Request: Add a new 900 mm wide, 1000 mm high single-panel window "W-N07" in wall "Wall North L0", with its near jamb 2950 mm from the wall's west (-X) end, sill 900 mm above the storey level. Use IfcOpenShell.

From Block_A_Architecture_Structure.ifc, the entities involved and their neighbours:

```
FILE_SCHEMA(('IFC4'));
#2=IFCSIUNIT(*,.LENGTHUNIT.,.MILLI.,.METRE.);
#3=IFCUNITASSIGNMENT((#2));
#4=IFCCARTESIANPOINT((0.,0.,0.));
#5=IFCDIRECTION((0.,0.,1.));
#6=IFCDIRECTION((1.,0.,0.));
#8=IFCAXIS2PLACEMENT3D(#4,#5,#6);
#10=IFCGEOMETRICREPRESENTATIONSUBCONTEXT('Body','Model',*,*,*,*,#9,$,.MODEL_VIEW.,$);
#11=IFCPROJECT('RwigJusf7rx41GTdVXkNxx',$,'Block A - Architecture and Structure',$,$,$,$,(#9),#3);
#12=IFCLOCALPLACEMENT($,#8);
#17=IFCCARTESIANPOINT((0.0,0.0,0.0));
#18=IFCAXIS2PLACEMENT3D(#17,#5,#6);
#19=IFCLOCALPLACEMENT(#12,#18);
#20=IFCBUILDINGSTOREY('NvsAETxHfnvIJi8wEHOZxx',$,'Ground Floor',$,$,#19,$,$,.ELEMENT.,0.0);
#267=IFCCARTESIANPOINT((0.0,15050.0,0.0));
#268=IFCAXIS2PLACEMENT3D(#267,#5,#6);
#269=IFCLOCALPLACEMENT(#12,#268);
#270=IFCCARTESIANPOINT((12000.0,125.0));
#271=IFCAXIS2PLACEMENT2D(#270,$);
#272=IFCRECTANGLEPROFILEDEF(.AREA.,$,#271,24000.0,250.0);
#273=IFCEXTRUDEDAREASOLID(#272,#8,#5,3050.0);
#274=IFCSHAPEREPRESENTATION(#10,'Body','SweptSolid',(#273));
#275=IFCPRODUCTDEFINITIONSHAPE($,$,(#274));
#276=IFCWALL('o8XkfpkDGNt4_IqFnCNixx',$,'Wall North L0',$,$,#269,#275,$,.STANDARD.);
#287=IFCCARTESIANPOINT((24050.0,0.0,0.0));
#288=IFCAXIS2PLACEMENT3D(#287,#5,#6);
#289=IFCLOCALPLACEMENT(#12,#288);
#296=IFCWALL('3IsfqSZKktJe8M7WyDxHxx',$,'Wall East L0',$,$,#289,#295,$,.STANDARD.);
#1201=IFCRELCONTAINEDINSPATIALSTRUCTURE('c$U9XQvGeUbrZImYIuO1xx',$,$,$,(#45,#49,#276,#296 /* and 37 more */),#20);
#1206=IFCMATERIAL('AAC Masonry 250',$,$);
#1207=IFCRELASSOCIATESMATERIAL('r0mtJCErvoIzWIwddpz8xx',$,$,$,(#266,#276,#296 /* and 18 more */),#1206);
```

```python
import numpy as np
import ifcopenshell
import ifcopenshell.api.feature
import ifcopenshell.api.geometry
import ifcopenshell.api.root
import ifcopenshell.api.spatial
import ifcopenshell.geom
import ifcopenshell.util.element
import ifcopenshell.util.placement
import ifcopenshell.util.representation
import ifcopenshell.util.shape
import ifcopenshell.util.unit

model = ifcopenshell.open("Block_A_Architecture_Structure.ifc")
unit_scale = ifcopenshell.util.unit.calculate_unit_scale(model)
settings = ifcopenshell.geom.settings()


def volume(element):
    """Net volume in cubic metres, openings subtracted."""
    shape = ifcopenshell.geom.create_shape(settings, element)
    return ifcopenshell.util.shape.get_volume(shape.geometry)


wall = model.by_guid("o8XkfpkDGNt4_IqFnCNixx")
storey = ifcopenshell.util.element.get_container(wall, ifc_class="IfcBuildingStorey")
context = ifcopenshell.util.representation.get_context(model, "Model", "Body", "MODEL_VIEW")
before = volume(wall)

width, height, from_end, sill = 0.9, 1, 2.95, 0.9  # metres

# The wall runs along its own X axis, and the end named is its -X end.
wall_shape = ifcopenshell.geom.create_shape(settings, wall)
x, y, z = ifcopenshell.util.shape.get_vertices(wall_shape.geometry).T
start = x.min() + from_end
face, thickness = float(y.min()), float(y.max() - y.min())
wall_matrix = ifcopenshell.util.placement.get_local_placement(wall.ObjectPlacement)
level = ifcopenshell.util.placement.get_local_placement(storey.ObjectPlacement)[2, 3]


def in_wall(x, y):
    """Placement at x, y metres in the wall's axes, at sill height."""
    matrix = wall_matrix.copy()
    matrix[:, 3] = wall_matrix @ np.array([x / unit_scale, y / unit_scale, 0.0, 1.0])
    matrix[2, 3] = level + sill / unit_scale
    return matrix


# Opening: a box that overshoots both wall faces by 50 mm.
opening = ifcopenshell.api.root.create_entity(model, ifc_class="IfcOpeningElement", predefined_type="OPENING")
box = ifcopenshell.api.geometry.add_wall_representation(
    model, context=context, length=width, height=height, thickness=thickness + 0.1
)
ifcopenshell.api.geometry.assign_representation(model, product=opening, representation=box)
ifcopenshell.api.geometry.edit_object_placement(model, product=opening, matrix=in_wall(start, face - 0.05), is_si=False)
ifcopenshell.api.feature.add_feature(model, feature=opening, element=wall)

window = ifcopenshell.api.root.create_entity(model, ifc_class="IfcWindow", name="W-N07", predefined_type="WINDOW")
window.OverallWidth, window.OverallHeight = width / unit_scale, height / unit_scale
window.PartitioningType = "SINGLE_PANEL"
body = ifcopenshell.api.geometry.add_window_representation(
    model,
    context=context,
    overall_width=window.OverallWidth,
    overall_height=window.OverallHeight,
    partition_type="SINGLE_PANEL",
)
ifcopenshell.api.geometry.assign_representation(model, product=window, representation=body)
ifcopenshell.api.spatial.assign_container(model, products=[window], relating_structure=storey)
ifcopenshell.api.feature.add_filling(model, opening=opening, element=window)

# Centre the window in the wall's thickness.
ifcopenshell.api.geometry.edit_object_placement(model, product=window, matrix=in_wall(start, face), is_si=False)
window_shape = ifcopenshell.geom.create_shape(settings, window)
depth = ifcopenshell.util.shape.get_vertices(window_shape.geometry)[:, 1]
offset = face + thickness / 2 - (depth.min() + depth.max()) / 2
ifcopenshell.api.geometry.edit_object_placement(model, product=window, matrix=in_wall(start, offset), is_si=False)

after = volume(wall)

print(f"wall volume {before:.3f} -> {after:.3f} m3")

model.write("Block_A_Architecture_Structure_rev.ifc")
```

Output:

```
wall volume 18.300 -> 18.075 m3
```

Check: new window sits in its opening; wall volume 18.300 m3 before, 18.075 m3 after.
